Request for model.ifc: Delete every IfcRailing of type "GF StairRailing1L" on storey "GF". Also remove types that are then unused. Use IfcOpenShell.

First a look at what the model holds.

```python
import ifcopenshell
import ifcopenshell.util.element

model = ifcopenshell.open("model.ifc")
print(model.schema)
storey = next(s for s in model.by_type("IfcBuildingStorey") if s.Name == "GF")
railings = [e for e in ifcopenshell.util.element.get_decomposition(storey) if e.is_a("IfcRailing")]
seen = {}
for e in railings:
    element_type = ifcopenshell.util.element.get_type(e)
    name = element_type.Name if element_type not in (None, e) else None
    seen[name] = seen.get(name, 0) + 1
for name, count in sorted(seen.items(), key=str):
    print(count, "x", name)
```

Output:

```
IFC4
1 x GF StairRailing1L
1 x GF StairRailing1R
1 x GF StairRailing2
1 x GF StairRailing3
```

```python
import ifcopenshell
import ifcopenshell.api.root
import ifcopenshell.util.element

model = ifcopenshell.open("model.ifc")

storey = next(s for s in model.by_type("IfcBuildingStorey") if s.Name == "GF")
railings = [e for e in ifcopenshell.util.element.get_decomposition(storey) if e.is_a("IfcRailing")]
targets = [e for e in railings if (t := ifcopenshell.util.element.get_type(e)) not in (None, e) and t.Name == "GF StairRailing1L"]
types = {ifcopenshell.util.element.get_type(e) for e in targets} - {None, *targets}

for e in targets:
    ifcopenshell.api.root.remove_product(model, product=e)
print(len(targets), "removed")

unused = [t for t in types if not ifcopenshell.util.element.get_types(t)]
for t in unused:
    ifcopenshell.api.root.remove_product(model, product=t)
print(len(unused), "unused types removed")

model.write("model_v2.ifc")
```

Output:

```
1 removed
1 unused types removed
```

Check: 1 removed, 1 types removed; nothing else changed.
